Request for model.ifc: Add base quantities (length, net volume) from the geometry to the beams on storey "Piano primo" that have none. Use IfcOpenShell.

First a look at what the model holds.

```python
import ifcopenshell
import ifcopenshell.util.element
import ifcopenshell.util.unit

model = ifcopenshell.open("model.ifc")
print(model.schema)
for unit_type in ("LENGTHUNIT", "AREAUNIT", "VOLUMEUNIT"):
    print(unit_type, ifcopenshell.util.unit.calculate_unit_scale(model, unit_type))
storey = next(s for s in model.by_type("IfcBuildingStorey") if s.Name == "Piano primo")
beams = [e for e in ifcopenshell.util.element.get_decomposition(storey) if e.is_a("IfcBeam")]
for e in sorted(beams, key=lambda e: e.id()):
    print(e.id(), e.is_a(), e.Name, list(ifcopenshell.util.element.get_psets(e, qtos_only=True)), sep=" | ")
```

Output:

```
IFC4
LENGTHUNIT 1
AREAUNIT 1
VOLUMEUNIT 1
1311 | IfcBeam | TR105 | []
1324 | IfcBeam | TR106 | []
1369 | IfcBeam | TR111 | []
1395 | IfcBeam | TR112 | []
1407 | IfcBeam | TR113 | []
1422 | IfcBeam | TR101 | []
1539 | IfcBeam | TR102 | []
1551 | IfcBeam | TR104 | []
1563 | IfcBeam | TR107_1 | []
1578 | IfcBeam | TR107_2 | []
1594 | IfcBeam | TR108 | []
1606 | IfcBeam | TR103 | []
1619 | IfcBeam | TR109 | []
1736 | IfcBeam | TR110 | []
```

```python
import ifcopenshell
import ifcopenshell.api.pset
import ifcopenshell.geom
import ifcopenshell.util.element
import ifcopenshell.util.shape
import ifcopenshell.util.unit

model = ifcopenshell.open("model.ifc")
unit_scale = ifcopenshell.util.unit.calculate_unit_scale(model)
volume_scale = ifcopenshell.util.unit.calculate_unit_scale(model, "VOLUMEUNIT")
settings = ifcopenshell.geom.settings()

storey = next(s for s in model.by_type("IfcBuildingStorey") if s.Name == "Piano primo")
beams = [e for e in ifcopenshell.util.element.get_decomposition(storey) if e.is_a("IfcBeam")]

for e in sorted(beams, key=lambda e: e.id()):
    if ifcopenshell.util.element.get_psets(e, qtos_only=True, should_inherit=False):
        continue
    # Geometry comes back in metres, in the element's own axes.
    shape = ifcopenshell.geom.create_shape(settings, e)
    values = {
        "Length": ifcopenshell.util.shape.get_max_xyz(shape.geometry) / unit_scale,
        "NetVolume": ifcopenshell.util.shape.get_volume(shape.geometry) / volume_scale,
    }
    qto = ifcopenshell.api.pset.add_qto(model, product=e, name="Qto_BeamBaseQuantities")
    ifcopenshell.api.pset.edit_qto(model, qto=qto, properties=values)
    print(e.id(), {k: round(v, 3) for k, v in values.items()})

model.write("model_updated.ifc")
```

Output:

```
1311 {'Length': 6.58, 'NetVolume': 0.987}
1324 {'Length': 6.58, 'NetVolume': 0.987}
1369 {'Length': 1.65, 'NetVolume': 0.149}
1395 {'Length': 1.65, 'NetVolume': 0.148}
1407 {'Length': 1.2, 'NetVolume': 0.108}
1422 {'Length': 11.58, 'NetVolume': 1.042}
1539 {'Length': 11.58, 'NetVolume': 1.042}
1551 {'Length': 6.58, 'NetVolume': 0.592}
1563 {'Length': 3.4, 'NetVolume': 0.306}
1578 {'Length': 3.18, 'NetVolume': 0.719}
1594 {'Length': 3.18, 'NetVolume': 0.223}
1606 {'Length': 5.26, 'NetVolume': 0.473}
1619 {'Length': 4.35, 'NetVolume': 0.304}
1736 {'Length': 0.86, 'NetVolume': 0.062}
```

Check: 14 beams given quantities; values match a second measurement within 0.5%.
